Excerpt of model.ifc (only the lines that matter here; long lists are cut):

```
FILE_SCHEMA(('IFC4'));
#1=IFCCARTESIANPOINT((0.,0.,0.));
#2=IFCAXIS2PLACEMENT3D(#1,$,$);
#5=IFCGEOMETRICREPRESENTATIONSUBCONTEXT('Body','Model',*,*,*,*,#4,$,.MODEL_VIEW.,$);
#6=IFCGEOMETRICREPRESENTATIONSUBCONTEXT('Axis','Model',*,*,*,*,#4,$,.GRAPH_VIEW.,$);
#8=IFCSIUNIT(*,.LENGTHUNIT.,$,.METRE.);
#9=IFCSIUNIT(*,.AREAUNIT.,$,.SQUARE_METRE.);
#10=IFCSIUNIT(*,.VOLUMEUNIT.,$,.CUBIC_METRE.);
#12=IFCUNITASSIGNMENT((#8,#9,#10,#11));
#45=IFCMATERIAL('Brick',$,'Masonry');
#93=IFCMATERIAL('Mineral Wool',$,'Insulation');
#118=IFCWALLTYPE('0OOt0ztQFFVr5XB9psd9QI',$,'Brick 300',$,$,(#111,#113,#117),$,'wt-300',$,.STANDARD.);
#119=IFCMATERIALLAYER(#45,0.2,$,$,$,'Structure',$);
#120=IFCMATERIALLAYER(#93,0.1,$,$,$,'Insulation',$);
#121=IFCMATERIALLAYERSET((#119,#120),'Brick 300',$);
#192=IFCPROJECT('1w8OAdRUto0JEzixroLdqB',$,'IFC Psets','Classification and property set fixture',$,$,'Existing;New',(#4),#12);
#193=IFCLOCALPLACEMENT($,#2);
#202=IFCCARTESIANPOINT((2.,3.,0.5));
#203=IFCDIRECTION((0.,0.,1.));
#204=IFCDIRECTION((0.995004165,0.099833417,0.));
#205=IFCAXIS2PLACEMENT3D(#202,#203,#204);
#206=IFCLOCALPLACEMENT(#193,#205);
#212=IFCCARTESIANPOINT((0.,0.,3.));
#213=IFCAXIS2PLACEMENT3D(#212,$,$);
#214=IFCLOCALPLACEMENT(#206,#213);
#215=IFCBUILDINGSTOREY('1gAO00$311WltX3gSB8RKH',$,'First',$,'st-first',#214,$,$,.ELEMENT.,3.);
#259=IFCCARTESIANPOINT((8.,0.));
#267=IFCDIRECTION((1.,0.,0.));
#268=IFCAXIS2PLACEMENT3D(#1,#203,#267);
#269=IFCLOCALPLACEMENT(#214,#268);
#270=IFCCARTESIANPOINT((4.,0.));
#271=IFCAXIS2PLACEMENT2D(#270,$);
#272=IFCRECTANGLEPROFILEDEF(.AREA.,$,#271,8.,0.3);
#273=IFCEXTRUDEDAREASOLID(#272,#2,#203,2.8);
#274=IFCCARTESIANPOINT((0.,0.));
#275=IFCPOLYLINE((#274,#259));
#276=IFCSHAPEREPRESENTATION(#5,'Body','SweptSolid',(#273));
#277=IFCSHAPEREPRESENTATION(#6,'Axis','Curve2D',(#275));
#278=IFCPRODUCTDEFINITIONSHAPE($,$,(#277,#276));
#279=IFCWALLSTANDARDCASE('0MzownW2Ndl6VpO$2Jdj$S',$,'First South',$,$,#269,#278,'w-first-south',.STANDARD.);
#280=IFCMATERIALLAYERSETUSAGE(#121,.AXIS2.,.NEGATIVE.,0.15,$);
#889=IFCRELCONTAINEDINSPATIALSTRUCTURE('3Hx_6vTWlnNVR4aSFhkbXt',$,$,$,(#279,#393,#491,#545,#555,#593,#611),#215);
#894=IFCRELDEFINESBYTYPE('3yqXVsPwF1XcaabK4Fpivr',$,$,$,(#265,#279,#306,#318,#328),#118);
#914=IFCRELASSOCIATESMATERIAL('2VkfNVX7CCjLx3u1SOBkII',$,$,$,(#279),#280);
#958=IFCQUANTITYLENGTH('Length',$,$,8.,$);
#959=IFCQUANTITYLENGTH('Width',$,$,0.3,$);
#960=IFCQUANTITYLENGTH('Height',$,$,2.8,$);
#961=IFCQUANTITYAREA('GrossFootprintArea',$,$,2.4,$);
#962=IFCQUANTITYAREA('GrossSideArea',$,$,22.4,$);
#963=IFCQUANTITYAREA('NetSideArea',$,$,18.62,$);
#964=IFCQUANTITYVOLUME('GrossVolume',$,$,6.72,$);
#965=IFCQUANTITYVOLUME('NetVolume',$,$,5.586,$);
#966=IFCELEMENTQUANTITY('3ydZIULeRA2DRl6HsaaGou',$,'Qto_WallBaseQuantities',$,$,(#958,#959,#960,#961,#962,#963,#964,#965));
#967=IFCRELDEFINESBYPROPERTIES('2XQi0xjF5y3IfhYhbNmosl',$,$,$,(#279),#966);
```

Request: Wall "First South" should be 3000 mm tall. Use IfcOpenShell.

```python
import ifcopenshell
import ifcopenshell.api.pset
import ifcopenshell.geom
import ifcopenshell.util.element
import ifcopenshell.util.representation
import ifcopenshell.util.shape
import ifcopenshell.util.unit

model = ifcopenshell.open("model.ifc")
unit_scale = ifcopenshell.util.unit.calculate_unit_scale(model)
area_scale = ifcopenshell.util.unit.calculate_unit_scale(model, "AREAUNIT")
volume_scale = ifcopenshell.util.unit.calculate_unit_scale(model, "VOLUMEUNIT")
settings = ifcopenshell.geom.settings()


def volume(element):
    """Net volume in cubic metres, openings subtracted."""
    shape = ifcopenshell.geom.create_shape(settings, element)
    return ifcopenshell.util.shape.get_volume(shape.geometry)


wall = model.by_guid("0MzownW2Ndl6VpO$2Jdj$S")
before = volume(wall)

body = ifcopenshell.util.representation.get_representation(wall, "Model", "Body")
solid = body.Items[0]
old_height = solid.Depth
solid.Depth = 3.0
after = volume(wall)
thickness = 0.3  # wall thickness in metres

# Update the stored height, areas and volumes.
qto = model.by_id(ifcopenshell.util.element.get_pset(wall, "Qto_WallBaseQuantities", should_inherit=False)["id"])
ifcopenshell.api.pset.edit_qto(model, qto=qto, properties={
    "Height": solid.Depth,
    "GrossSideArea": ifcopenshell.util.element.get_pset(wall, "Qto_WallBaseQuantities", "GrossSideArea") * solid.Depth / old_height,
    "NetSideArea": after / thickness / area_scale,
    "GrossVolume": ifcopenshell.util.element.get_pset(wall, "Qto_WallBaseQuantities", "GrossVolume") * solid.Depth / old_height,
    "NetVolume": after / volume_scale,
})

print(f"height {old_height:g} -> {solid.Depth:g}, volume {before:.3f} -> {after:.3f} m3")

model.write("model_rev.ifc")
```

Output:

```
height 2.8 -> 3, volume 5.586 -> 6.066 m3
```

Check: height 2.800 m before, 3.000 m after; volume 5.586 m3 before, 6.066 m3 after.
